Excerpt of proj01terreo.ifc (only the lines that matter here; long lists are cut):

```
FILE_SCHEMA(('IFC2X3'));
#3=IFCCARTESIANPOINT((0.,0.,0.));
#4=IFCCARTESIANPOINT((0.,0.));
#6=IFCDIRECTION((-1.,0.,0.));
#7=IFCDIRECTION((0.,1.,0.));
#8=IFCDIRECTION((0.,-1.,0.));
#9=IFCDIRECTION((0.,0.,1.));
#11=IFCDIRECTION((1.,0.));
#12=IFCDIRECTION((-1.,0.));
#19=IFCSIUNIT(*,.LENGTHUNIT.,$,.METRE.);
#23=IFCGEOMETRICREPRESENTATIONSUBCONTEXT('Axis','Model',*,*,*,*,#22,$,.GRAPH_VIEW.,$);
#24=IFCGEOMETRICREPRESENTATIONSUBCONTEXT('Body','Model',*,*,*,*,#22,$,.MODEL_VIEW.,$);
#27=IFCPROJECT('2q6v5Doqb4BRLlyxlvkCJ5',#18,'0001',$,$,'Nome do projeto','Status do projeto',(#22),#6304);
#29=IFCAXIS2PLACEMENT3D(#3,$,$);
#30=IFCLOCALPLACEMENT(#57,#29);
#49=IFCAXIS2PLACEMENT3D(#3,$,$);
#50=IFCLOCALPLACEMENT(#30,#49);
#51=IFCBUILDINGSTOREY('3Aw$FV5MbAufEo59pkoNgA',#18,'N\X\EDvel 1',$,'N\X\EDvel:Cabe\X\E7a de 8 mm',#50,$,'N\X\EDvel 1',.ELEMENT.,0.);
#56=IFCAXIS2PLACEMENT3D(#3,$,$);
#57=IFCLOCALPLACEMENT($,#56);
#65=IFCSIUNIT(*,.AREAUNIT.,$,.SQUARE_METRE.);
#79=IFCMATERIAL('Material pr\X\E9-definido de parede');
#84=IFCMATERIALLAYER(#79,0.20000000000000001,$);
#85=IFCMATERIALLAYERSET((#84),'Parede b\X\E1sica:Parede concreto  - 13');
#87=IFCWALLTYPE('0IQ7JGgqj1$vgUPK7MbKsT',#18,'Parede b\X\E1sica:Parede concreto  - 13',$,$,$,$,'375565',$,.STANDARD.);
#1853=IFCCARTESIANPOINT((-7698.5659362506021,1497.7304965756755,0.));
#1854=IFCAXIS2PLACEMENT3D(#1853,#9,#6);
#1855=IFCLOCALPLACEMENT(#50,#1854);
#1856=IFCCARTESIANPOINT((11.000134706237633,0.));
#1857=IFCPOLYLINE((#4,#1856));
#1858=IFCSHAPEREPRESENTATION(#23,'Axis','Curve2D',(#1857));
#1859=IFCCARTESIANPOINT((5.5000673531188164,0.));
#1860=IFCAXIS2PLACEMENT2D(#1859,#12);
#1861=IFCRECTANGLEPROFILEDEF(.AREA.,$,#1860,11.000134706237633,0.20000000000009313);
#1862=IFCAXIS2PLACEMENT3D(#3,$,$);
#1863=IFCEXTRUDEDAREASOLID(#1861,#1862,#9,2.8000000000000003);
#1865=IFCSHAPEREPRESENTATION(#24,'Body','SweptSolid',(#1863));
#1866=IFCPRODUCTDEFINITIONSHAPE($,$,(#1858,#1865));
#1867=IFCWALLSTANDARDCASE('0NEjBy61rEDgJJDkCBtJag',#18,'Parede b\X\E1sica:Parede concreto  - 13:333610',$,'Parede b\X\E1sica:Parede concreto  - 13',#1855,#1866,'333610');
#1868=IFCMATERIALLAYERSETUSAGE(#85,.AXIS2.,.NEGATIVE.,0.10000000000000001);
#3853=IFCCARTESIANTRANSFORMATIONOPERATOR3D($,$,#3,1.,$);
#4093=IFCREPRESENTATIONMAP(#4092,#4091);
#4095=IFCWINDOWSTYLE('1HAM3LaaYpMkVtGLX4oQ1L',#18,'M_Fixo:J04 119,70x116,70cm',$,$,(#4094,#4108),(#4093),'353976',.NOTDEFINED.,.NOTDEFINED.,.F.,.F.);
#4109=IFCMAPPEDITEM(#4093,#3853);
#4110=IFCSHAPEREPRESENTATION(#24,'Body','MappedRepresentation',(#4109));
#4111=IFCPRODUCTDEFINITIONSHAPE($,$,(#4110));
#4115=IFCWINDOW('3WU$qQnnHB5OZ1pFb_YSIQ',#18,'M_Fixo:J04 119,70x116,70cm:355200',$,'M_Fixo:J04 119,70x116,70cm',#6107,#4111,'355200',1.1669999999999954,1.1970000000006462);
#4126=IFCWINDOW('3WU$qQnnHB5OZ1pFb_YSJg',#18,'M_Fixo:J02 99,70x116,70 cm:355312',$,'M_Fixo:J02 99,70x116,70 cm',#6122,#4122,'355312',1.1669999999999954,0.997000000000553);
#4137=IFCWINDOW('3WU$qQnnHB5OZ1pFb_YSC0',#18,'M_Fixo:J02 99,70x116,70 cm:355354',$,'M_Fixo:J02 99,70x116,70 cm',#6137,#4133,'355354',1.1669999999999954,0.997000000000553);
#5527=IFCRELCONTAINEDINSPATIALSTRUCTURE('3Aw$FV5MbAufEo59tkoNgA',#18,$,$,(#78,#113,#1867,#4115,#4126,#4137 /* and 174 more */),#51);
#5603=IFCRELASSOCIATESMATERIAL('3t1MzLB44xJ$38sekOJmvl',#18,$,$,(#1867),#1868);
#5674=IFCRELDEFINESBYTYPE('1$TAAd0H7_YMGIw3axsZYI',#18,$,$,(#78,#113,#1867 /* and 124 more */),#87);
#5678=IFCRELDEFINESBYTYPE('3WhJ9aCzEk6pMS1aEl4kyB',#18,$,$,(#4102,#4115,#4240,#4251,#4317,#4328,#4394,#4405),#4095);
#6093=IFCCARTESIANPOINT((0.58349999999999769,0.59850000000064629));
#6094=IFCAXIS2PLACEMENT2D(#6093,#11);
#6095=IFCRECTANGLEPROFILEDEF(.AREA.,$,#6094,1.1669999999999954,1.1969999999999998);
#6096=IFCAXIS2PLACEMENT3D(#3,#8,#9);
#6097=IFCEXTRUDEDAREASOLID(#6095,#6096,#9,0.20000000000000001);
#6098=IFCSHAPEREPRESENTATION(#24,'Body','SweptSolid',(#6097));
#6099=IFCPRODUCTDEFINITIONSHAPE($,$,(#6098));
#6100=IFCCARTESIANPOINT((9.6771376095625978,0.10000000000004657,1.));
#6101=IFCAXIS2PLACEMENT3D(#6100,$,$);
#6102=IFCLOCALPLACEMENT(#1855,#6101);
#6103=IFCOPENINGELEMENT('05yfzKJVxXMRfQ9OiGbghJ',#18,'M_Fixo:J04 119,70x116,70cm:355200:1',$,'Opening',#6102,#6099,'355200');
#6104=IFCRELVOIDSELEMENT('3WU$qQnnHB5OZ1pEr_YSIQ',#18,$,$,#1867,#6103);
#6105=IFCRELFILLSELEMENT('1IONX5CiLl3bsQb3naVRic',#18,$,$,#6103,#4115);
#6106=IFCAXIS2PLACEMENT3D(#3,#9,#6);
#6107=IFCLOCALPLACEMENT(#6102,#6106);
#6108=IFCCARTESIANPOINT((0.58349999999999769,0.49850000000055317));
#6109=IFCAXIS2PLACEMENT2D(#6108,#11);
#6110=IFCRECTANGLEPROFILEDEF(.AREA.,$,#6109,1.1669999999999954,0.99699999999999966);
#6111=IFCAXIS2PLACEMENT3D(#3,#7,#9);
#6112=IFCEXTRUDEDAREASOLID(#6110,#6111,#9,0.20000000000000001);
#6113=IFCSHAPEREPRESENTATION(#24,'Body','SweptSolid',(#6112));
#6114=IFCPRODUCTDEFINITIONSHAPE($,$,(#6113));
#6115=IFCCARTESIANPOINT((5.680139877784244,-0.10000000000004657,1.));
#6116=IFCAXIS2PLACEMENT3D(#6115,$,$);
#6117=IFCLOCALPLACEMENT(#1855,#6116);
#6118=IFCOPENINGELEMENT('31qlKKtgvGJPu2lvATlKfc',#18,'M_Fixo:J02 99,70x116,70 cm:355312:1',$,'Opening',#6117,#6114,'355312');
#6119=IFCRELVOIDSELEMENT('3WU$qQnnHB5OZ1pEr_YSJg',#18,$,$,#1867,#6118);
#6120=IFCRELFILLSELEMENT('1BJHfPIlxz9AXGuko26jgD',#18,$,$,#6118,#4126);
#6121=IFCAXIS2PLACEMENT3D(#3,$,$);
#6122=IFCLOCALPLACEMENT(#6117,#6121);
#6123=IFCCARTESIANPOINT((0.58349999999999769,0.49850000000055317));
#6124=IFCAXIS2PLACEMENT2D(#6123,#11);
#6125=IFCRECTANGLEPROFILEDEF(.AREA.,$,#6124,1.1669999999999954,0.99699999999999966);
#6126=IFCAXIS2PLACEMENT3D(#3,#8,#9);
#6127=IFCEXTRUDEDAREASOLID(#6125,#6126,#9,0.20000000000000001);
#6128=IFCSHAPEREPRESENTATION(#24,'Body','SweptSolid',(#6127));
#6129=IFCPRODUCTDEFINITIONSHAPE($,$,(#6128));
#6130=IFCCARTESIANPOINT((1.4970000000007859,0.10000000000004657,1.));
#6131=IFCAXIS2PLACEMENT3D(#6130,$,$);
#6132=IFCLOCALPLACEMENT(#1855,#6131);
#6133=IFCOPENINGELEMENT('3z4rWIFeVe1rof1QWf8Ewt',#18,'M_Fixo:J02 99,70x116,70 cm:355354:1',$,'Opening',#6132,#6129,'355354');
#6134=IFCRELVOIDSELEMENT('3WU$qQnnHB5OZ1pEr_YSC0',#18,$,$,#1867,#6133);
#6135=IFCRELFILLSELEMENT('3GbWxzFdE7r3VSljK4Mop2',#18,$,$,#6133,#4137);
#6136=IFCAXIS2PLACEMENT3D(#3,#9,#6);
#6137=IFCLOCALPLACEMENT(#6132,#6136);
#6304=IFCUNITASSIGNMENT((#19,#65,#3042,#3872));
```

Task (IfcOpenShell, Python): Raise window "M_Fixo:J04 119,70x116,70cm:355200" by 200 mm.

```python
import numpy as np
import ifcopenshell
import ifcopenshell.api.geometry
import ifcopenshell.util.placement
import ifcopenshell.util.unit

model = ifcopenshell.open("proj01terreo.ifc")
unit_scale = ifcopenshell.util.unit.calculate_unit_scale(model)

window = model.by_guid("3WU$qQnnHB5OZ1pFb_YSIQ")
opening = window.FillsVoids[0].RelatingOpeningElement
dz = 0.2 / unit_scale

shift = np.array([0.0, 0.0, dz])
# The window is placed relative to its opening, so it follows when the opening moves.
matrix = ifcopenshell.util.placement.get_local_placement(opening.ObjectPlacement)
matrix[:3, 3] += shift
ifcopenshell.api.geometry.edit_object_placement(
    model, product=opening, matrix=matrix, is_si=False, should_transform_children=True
)

print(f"moved by {dz * unit_scale:+.3f} m")

model.write("proj01terreo_edited.ifc")
```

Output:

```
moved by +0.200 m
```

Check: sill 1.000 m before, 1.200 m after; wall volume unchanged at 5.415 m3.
